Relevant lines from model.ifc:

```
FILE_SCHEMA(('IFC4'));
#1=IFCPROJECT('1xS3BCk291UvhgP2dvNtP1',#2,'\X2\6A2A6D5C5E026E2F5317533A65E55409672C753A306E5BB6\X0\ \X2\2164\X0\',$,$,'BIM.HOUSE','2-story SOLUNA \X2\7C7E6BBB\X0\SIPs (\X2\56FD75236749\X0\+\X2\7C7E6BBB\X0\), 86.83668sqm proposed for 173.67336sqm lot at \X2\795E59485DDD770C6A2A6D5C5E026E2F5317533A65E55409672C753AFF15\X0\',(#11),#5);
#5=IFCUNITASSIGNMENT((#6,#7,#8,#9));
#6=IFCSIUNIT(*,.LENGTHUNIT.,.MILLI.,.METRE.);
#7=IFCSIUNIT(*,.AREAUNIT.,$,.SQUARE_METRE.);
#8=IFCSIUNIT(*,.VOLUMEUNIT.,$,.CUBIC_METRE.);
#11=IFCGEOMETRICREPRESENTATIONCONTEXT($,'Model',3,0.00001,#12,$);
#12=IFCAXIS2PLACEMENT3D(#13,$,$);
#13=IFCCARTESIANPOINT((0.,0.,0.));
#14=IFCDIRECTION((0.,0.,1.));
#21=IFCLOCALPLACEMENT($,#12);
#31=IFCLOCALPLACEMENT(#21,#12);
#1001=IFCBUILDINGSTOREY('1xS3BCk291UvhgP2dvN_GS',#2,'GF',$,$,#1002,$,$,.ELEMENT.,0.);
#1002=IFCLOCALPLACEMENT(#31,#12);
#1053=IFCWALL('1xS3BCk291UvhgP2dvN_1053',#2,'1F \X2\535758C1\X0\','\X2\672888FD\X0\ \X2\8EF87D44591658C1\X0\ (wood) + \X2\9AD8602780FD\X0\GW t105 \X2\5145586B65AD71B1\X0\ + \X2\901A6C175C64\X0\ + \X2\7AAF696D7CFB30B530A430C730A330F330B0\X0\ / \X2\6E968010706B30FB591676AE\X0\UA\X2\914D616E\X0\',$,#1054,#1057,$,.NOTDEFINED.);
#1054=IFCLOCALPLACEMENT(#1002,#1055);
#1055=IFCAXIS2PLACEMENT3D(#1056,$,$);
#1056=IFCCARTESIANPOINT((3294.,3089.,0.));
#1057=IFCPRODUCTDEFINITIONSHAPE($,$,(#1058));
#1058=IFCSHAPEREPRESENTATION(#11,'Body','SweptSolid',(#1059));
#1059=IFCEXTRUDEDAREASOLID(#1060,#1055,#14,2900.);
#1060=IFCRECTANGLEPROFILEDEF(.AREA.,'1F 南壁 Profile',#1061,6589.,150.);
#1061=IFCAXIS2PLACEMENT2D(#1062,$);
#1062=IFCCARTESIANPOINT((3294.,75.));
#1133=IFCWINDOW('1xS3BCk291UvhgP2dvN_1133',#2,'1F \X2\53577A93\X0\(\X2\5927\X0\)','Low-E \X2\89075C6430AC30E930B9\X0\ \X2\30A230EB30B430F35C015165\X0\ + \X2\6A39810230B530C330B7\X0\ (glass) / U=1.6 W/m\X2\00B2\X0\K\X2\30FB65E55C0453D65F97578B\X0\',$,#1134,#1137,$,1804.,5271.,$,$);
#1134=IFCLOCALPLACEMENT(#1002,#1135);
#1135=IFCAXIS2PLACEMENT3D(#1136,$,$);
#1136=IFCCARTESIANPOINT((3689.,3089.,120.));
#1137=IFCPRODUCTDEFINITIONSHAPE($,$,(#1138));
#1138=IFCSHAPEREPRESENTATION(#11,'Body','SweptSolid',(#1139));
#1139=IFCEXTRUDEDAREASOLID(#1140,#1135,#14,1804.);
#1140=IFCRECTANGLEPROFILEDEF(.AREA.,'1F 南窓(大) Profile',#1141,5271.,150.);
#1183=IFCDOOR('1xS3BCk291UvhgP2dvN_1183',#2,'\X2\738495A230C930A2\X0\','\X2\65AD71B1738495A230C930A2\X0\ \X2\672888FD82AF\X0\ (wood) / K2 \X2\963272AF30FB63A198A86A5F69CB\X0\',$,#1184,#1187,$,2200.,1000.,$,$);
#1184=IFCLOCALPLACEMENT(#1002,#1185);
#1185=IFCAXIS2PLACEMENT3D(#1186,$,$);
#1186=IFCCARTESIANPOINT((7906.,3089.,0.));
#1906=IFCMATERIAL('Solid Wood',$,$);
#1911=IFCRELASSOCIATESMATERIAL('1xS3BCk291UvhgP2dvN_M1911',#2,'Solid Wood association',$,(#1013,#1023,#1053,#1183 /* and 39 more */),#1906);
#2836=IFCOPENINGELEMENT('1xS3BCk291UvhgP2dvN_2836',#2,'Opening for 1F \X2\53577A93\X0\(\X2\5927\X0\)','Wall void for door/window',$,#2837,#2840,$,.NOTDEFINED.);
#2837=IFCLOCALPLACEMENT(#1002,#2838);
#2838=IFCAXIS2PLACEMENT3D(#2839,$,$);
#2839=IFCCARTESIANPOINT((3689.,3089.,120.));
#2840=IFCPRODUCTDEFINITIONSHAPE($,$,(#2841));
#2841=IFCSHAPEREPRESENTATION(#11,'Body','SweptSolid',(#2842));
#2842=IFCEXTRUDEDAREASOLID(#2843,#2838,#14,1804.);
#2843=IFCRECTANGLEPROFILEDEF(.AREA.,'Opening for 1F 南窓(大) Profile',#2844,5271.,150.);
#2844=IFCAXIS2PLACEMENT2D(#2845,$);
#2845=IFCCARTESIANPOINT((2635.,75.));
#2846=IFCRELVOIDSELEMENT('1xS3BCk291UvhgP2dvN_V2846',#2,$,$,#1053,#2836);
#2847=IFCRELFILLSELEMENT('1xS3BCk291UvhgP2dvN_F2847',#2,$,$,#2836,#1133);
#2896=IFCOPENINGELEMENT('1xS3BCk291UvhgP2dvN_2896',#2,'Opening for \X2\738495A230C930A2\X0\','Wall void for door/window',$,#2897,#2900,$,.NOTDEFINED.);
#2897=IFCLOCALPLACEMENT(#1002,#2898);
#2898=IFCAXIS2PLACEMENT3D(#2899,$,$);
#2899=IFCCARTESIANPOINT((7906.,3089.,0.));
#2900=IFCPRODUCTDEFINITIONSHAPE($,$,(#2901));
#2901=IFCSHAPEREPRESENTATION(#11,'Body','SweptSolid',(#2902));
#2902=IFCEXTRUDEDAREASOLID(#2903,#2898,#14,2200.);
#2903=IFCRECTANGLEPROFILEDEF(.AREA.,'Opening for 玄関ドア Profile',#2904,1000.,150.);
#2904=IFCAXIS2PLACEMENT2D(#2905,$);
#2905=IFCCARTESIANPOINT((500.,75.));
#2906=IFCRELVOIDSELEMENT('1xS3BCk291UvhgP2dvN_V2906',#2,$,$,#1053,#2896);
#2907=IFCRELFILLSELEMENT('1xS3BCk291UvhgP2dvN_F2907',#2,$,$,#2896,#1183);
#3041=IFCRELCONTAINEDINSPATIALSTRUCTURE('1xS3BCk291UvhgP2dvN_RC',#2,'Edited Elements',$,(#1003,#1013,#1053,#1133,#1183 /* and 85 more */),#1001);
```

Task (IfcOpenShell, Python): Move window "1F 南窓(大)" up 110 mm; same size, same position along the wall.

```python
import numpy as np
import ifcopenshell
import ifcopenshell.api.geometry
import ifcopenshell.util.placement
import ifcopenshell.util.unit

model = ifcopenshell.open("model.ifc")
unit_scale = ifcopenshell.util.unit.calculate_unit_scale(model)

window = model.by_guid("1xS3BCk291UvhgP2dvN_1133")
opening = window.FillsVoids[0].RelatingOpeningElement
dz = 0.11 / unit_scale

shift = np.array([0.0, 0.0, dz])
# The window is not placed relative to its opening, so move both.
for product in (opening, window):
    matrix = ifcopenshell.util.placement.get_local_placement(product.ObjectPlacement)
    matrix[:3, 3] += shift
    ifcopenshell.api.geometry.edit_object_placement(model, product=product, matrix=matrix, is_si=False)

print(f"moved by {dz * unit_scale:+.3f} m")

model.write("model_v2.ifc")
```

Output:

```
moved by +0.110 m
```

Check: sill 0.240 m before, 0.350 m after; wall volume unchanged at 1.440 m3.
